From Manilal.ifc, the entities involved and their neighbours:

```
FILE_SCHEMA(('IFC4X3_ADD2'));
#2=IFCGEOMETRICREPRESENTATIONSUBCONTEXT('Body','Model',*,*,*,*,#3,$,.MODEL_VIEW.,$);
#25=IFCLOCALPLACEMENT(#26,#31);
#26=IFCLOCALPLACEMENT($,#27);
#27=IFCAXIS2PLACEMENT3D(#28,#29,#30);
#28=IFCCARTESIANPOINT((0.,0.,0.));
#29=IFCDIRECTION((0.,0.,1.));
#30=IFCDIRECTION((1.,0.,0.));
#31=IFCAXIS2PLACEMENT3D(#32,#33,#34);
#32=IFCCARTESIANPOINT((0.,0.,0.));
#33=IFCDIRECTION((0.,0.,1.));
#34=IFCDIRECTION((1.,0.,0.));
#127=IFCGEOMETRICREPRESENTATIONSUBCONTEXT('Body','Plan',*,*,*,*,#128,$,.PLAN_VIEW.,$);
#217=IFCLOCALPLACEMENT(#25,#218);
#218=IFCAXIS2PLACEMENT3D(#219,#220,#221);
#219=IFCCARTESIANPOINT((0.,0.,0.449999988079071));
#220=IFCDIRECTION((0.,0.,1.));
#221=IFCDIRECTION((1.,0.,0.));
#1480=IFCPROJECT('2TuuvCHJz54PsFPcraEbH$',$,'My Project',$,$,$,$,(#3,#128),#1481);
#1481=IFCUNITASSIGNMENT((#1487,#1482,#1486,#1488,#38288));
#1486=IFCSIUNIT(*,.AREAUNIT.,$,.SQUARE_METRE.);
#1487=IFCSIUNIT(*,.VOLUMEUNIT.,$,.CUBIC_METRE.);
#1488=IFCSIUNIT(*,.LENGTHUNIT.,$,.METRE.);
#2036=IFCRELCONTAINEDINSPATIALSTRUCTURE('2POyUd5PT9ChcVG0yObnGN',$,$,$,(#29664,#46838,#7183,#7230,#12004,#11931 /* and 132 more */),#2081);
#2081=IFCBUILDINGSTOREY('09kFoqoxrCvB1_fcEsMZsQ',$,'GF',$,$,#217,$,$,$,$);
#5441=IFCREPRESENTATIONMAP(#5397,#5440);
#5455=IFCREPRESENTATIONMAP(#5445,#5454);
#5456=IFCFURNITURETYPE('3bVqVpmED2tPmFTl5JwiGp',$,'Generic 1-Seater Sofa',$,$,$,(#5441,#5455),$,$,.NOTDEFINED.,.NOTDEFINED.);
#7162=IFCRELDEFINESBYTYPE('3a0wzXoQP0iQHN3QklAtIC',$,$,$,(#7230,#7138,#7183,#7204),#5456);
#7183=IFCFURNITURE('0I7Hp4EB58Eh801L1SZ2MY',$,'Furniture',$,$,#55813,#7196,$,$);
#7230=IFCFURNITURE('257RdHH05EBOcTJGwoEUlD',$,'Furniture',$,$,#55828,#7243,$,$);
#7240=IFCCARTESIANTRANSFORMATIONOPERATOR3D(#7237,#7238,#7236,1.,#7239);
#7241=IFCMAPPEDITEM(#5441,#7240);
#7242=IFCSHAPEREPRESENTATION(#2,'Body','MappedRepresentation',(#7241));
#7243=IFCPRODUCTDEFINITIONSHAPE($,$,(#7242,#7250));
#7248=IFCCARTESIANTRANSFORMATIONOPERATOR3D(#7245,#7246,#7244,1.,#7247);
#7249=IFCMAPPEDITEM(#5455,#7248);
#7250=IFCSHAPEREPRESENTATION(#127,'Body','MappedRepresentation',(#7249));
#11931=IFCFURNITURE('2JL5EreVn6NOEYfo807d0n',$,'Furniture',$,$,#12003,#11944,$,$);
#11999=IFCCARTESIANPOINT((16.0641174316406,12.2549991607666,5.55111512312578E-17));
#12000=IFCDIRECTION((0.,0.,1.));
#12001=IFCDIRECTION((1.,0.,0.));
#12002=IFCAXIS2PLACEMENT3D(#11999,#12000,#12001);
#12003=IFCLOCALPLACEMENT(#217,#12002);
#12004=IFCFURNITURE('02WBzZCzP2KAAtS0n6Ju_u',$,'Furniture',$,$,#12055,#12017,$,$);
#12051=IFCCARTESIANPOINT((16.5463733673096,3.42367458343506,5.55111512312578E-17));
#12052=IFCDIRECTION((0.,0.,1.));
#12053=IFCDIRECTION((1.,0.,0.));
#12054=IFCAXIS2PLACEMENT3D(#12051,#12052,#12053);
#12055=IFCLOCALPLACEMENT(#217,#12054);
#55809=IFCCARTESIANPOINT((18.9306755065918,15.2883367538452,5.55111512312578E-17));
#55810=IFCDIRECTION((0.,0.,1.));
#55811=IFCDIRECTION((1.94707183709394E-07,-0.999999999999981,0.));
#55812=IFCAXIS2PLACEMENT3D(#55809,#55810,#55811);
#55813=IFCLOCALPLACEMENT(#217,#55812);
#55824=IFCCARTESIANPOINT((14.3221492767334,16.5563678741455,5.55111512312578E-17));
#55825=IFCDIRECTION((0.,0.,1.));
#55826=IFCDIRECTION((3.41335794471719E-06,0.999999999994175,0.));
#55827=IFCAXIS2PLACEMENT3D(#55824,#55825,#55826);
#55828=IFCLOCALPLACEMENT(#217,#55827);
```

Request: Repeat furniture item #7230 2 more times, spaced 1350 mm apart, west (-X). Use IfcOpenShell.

```python
import numpy as np
import ifcopenshell
import ifcopenshell.api.geometry
import ifcopenshell.api.root
import ifcopenshell.util.element
import ifcopenshell.util.placement
import ifcopenshell.util.unit

model = ifcopenshell.open("Manilal.ifc")
unit_scale = ifcopenshell.util.unit.calculate_unit_scale(model)

source = model.by_guid("257RdHH05EBOcTJGwoEUlD")
base = ifcopenshell.util.placement.get_local_placement(source.ObjectPlacement)
step = np.array([-1.0, 0.0, 0.0]) * 1.35 / unit_scale

for i in range(1, 3):
    copy = ifcopenshell.api.root.copy_class(model, product=source)
    copy.Representation = ifcopenshell.util.element.copy_deep(
        model, source.Representation, exclude=["IfcGeometricRepresentationContext", "IfcRepresentationMap"]
    )
    matrix = base.copy()
    matrix[:3, 3] += i * step
    print("added at", matrix[:3, 3].round(3) + 0.0)
    ifcopenshell.api.geometry.edit_object_placement(model, product=copy, matrix=matrix, is_si=False)

model.write("Manilal-out.ifc")
```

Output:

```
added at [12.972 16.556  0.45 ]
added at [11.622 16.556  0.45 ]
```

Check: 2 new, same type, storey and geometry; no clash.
